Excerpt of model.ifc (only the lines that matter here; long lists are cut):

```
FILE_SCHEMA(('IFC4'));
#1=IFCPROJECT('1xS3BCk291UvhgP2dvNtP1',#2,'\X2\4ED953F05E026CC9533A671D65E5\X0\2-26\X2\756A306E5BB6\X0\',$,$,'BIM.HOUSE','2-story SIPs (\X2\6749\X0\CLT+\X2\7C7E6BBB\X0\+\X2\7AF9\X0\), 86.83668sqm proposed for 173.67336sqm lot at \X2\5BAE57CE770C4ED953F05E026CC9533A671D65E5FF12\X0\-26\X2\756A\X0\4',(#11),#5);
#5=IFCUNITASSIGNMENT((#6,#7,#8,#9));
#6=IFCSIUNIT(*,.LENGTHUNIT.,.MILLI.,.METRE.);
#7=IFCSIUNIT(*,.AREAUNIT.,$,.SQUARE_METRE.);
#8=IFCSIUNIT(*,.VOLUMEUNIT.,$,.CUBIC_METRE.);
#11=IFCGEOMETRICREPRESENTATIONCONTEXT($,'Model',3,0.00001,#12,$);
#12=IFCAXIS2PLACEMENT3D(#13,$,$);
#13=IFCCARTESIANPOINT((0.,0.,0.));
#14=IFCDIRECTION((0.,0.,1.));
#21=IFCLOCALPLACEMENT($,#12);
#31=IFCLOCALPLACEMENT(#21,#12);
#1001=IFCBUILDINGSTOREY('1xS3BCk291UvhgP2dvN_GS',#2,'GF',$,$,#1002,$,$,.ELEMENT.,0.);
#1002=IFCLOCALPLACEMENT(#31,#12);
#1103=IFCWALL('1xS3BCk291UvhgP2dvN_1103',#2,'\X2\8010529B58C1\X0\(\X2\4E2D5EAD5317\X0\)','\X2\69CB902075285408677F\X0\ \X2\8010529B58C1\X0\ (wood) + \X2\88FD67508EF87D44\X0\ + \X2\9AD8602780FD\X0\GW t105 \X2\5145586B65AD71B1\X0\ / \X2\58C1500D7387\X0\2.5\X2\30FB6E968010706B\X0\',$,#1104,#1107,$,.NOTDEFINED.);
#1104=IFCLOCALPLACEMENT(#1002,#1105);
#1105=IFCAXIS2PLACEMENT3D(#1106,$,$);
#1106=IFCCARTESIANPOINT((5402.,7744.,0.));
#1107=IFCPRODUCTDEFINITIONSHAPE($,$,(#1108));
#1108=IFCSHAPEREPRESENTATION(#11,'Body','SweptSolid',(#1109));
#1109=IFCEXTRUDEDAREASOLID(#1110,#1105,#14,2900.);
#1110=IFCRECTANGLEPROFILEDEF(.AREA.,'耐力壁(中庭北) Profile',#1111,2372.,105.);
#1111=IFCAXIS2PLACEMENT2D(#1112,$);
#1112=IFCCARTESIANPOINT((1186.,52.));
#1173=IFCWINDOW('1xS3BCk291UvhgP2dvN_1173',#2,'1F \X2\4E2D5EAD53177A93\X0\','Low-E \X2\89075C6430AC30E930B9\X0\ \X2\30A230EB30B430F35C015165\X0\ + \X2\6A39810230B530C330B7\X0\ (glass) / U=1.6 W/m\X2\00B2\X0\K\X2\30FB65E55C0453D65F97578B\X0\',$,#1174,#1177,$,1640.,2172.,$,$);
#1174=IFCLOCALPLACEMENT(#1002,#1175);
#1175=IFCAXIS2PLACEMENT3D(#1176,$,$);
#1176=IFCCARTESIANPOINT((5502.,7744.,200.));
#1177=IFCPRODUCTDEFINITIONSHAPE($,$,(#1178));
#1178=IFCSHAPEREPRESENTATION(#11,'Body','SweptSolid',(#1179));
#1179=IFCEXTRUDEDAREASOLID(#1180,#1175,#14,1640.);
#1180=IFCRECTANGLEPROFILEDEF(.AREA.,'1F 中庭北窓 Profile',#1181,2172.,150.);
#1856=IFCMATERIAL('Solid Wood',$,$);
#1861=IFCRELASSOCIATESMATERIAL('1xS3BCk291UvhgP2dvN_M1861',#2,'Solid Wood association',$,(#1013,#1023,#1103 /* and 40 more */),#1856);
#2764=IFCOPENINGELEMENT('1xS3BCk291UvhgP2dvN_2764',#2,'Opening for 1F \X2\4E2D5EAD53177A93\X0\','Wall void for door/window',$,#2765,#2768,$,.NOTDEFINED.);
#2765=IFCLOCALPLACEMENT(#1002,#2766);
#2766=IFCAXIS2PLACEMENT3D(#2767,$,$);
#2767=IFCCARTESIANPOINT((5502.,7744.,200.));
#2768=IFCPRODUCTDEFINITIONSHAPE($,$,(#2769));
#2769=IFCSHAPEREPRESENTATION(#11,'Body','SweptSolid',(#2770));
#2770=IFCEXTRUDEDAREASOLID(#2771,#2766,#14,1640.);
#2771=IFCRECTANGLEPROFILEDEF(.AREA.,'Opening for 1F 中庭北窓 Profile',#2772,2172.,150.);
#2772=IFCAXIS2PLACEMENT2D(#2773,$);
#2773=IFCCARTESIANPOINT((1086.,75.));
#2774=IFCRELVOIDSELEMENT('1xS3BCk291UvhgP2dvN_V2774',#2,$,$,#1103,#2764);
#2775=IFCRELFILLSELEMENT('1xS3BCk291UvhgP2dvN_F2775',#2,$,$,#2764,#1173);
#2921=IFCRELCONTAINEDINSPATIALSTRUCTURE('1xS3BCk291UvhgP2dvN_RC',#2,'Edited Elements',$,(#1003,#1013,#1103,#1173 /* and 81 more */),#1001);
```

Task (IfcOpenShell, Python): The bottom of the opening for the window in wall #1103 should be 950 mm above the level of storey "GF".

```python
import numpy as np
import ifcopenshell
import ifcopenshell.api.geometry
import ifcopenshell.geom
import ifcopenshell.util.element
import ifcopenshell.util.placement
import ifcopenshell.util.shape
import ifcopenshell.util.unit

model = ifcopenshell.open("model.ifc")
unit_scale = ifcopenshell.util.unit.calculate_unit_scale(model)

window = model.by_guid("1xS3BCk291UvhgP2dvN_1173")
opening = window.FillsVoids[0].RelatingOpeningElement
storey = ifcopenshell.util.element.get_container(window, ifc_class="IfcBuildingStorey")
level = ifcopenshell.util.placement.get_local_placement(storey.ObjectPlacement)[2, 3]

# The opening's origin need not be at the sill, so measure its lowest point.
shape = ifcopenshell.geom.create_shape(ifcopenshell.geom.settings(), opening)
bottom = ifcopenshell.util.shape.get_shape_bottom_elevation(shape, shape.geometry) / unit_scale
dz = level + 950.0 - bottom

shift = np.array([0.0, 0.0, dz])
# The window is not placed relative to its opening, so move both.
for product in (opening, window):
    matrix = ifcopenshell.util.placement.get_local_placement(product.ObjectPlacement)
    matrix[:3, 3] += shift
    ifcopenshell.api.geometry.edit_object_placement(model, product=product, matrix=matrix, is_si=False)

print(f"moved by {dz * unit_scale:+.3f} m")

model.write("model_v2.ifc")
```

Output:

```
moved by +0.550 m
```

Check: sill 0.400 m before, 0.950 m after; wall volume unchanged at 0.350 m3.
